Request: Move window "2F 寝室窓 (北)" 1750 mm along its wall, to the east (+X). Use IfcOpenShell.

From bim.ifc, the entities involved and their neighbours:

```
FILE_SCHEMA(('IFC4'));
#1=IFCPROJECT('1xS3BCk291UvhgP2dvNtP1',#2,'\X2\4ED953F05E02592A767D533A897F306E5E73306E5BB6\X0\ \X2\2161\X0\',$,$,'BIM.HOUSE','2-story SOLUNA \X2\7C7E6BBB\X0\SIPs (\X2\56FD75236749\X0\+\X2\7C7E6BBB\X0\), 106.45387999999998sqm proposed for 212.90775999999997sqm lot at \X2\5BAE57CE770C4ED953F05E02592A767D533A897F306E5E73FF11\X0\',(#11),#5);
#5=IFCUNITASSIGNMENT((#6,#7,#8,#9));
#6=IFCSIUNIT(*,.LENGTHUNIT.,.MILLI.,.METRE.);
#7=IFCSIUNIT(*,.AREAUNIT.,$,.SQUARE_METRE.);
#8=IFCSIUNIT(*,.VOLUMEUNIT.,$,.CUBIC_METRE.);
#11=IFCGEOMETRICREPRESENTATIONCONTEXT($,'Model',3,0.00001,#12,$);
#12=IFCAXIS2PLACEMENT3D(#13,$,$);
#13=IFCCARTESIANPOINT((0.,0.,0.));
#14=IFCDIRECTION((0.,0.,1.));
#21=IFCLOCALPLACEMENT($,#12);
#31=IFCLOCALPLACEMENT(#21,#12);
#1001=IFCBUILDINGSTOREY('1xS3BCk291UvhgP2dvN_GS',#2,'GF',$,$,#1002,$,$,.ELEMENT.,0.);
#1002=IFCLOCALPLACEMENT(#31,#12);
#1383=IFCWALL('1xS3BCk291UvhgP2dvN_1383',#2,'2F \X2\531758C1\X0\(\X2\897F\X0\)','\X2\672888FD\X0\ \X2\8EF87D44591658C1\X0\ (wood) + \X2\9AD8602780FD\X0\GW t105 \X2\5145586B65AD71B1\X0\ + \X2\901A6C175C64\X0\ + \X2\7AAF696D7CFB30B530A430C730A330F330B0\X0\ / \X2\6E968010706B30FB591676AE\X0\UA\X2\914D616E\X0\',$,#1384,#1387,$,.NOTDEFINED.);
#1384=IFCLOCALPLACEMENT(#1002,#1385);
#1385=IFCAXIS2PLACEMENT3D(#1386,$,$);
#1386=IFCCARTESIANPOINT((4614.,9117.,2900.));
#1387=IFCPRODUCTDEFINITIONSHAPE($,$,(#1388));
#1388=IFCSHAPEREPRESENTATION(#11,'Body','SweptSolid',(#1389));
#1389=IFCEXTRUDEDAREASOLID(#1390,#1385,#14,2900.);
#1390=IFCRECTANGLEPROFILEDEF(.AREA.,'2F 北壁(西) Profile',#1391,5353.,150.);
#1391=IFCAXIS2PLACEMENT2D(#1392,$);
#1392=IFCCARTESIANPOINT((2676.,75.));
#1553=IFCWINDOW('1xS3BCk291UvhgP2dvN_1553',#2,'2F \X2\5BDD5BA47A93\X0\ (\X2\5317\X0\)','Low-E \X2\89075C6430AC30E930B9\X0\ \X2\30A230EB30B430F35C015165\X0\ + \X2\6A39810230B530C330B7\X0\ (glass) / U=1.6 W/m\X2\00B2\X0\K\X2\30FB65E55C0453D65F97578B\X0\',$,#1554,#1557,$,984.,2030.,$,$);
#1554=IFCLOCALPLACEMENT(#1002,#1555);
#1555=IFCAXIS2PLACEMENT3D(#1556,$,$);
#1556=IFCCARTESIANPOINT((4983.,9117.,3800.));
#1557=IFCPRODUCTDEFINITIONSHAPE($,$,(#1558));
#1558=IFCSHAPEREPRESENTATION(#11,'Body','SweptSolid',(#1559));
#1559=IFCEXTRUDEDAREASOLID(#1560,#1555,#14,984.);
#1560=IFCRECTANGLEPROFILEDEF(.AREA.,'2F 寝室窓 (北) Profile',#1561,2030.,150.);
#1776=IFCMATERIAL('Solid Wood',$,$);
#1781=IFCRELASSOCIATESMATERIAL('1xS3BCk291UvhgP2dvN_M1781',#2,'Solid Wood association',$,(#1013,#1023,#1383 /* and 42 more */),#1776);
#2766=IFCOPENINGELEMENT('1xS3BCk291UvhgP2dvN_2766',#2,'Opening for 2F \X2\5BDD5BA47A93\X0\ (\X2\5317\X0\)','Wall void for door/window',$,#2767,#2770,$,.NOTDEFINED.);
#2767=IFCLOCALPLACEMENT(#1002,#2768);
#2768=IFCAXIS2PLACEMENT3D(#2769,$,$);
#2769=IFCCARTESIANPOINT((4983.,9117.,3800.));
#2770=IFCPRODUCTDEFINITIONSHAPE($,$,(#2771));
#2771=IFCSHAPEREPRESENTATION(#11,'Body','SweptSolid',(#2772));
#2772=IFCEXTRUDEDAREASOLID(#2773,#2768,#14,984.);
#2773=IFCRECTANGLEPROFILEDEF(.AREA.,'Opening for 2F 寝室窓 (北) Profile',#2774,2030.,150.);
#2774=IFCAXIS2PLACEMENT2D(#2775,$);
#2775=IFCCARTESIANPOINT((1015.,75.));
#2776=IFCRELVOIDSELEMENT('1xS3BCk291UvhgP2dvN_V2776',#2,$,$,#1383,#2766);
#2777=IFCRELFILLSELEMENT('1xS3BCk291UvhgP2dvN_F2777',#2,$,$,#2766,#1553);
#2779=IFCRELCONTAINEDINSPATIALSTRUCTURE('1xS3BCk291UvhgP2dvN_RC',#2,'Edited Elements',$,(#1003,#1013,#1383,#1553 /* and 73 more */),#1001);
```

```python
import ifcopenshell
import ifcopenshell.api.geometry
import ifcopenshell.util.placement
import ifcopenshell.util.unit

model = ifcopenshell.open("bim.ifc")
unit_scale = ifcopenshell.util.unit.calculate_unit_scale(model)

window = model.by_guid("1xS3BCk291UvhgP2dvN_1553")
opening = window.FillsVoids[0].RelatingOpeningElement
wall = opening.VoidsElements[0].RelatingBuildingElement

wall_matrix = ifcopenshell.util.placement.get_local_placement(wall.ObjectPlacement)
shift = wall_matrix[:3, 0] * 1.75 / unit_scale
before = ifcopenshell.util.placement.get_local_placement(window.ObjectPlacement)[:3, 3].copy()

# The window is not placed relative to its opening, so move both.
for product in (opening, window):
    matrix = ifcopenshell.util.placement.get_local_placement(product.ObjectPlacement)
    matrix[:3, 3] += shift
    ifcopenshell.api.geometry.edit_object_placement(model, product=product, matrix=matrix, is_si=False)

after = ifcopenshell.util.placement.get_local_placement(window.ObjectPlacement)[:3, 3]
print("window moved by", (after - before).round(3) + 0.0)

model.write("bim_edited.ifc")
```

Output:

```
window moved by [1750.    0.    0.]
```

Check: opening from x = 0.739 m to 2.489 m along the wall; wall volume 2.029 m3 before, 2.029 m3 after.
